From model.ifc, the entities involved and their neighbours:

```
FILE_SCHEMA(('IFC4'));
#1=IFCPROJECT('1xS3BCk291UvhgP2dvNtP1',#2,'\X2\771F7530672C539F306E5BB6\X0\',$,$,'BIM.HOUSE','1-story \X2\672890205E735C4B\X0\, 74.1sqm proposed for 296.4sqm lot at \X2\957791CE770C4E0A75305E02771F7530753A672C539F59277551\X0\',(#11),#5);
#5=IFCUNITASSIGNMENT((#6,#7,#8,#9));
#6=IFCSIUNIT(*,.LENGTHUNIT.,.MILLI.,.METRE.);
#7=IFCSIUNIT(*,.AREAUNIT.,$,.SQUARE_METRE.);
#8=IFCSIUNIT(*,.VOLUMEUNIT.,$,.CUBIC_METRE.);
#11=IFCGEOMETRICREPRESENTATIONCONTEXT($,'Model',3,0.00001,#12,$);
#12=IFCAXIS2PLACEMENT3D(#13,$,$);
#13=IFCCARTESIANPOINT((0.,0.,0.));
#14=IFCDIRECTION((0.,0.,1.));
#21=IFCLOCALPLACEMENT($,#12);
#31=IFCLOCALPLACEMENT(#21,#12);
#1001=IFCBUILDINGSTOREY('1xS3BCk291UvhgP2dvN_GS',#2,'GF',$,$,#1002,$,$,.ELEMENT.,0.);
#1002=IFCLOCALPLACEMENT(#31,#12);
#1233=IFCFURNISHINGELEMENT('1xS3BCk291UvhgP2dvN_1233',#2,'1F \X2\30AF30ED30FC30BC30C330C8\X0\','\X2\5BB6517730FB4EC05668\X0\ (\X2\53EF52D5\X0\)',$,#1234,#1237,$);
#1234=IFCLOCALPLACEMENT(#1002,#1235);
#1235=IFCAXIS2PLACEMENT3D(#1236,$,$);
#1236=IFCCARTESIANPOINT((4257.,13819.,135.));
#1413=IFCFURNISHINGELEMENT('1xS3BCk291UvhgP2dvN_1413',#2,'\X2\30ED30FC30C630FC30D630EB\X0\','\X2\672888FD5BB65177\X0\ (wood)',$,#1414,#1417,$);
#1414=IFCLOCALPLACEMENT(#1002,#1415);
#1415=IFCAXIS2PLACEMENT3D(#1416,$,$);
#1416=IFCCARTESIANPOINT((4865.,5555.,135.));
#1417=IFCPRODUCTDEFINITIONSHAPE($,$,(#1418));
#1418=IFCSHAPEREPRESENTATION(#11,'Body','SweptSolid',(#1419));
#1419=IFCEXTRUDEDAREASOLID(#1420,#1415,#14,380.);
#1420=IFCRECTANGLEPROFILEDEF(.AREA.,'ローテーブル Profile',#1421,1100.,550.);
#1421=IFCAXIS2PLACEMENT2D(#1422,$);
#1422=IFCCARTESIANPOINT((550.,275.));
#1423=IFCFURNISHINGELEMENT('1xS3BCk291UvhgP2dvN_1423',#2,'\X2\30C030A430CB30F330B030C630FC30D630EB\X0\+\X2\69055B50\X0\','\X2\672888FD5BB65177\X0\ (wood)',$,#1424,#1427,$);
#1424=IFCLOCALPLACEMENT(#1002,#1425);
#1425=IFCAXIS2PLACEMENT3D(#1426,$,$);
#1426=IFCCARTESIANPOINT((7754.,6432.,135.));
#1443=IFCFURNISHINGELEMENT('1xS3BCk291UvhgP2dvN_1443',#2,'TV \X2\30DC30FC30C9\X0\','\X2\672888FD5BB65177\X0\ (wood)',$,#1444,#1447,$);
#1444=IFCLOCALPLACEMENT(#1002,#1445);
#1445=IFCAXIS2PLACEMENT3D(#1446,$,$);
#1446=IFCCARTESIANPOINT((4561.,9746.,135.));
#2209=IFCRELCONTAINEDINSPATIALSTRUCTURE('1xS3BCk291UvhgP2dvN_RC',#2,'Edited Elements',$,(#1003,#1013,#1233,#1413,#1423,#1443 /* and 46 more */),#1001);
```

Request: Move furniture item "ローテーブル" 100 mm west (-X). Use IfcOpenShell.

```python
import ifcopenshell
import ifcopenshell.api.geometry
import ifcopenshell.util.placement
import ifcopenshell.util.unit

model = ifcopenshell.open("model.ifc")
unit_scale = ifcopenshell.util.unit.calculate_unit_scale(model)

item = model.by_guid("1xS3BCk291UvhgP2dvN_1413")
matrix = ifcopenshell.util.placement.get_local_placement(item.ObjectPlacement)
matrix[0, 3] -= 0.1 / unit_scale
ifcopenshell.api.geometry.edit_object_placement(model, product=item, matrix=matrix, is_si=False)

print(ifcopenshell.util.placement.get_local_placement(item.ObjectPlacement).round(3) + 0.0)

model.write("model_updated.ifc")
```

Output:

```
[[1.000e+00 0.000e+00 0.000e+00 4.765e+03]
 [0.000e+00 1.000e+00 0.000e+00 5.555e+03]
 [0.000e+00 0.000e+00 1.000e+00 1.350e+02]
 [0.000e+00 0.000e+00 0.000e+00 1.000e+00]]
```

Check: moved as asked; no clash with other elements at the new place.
